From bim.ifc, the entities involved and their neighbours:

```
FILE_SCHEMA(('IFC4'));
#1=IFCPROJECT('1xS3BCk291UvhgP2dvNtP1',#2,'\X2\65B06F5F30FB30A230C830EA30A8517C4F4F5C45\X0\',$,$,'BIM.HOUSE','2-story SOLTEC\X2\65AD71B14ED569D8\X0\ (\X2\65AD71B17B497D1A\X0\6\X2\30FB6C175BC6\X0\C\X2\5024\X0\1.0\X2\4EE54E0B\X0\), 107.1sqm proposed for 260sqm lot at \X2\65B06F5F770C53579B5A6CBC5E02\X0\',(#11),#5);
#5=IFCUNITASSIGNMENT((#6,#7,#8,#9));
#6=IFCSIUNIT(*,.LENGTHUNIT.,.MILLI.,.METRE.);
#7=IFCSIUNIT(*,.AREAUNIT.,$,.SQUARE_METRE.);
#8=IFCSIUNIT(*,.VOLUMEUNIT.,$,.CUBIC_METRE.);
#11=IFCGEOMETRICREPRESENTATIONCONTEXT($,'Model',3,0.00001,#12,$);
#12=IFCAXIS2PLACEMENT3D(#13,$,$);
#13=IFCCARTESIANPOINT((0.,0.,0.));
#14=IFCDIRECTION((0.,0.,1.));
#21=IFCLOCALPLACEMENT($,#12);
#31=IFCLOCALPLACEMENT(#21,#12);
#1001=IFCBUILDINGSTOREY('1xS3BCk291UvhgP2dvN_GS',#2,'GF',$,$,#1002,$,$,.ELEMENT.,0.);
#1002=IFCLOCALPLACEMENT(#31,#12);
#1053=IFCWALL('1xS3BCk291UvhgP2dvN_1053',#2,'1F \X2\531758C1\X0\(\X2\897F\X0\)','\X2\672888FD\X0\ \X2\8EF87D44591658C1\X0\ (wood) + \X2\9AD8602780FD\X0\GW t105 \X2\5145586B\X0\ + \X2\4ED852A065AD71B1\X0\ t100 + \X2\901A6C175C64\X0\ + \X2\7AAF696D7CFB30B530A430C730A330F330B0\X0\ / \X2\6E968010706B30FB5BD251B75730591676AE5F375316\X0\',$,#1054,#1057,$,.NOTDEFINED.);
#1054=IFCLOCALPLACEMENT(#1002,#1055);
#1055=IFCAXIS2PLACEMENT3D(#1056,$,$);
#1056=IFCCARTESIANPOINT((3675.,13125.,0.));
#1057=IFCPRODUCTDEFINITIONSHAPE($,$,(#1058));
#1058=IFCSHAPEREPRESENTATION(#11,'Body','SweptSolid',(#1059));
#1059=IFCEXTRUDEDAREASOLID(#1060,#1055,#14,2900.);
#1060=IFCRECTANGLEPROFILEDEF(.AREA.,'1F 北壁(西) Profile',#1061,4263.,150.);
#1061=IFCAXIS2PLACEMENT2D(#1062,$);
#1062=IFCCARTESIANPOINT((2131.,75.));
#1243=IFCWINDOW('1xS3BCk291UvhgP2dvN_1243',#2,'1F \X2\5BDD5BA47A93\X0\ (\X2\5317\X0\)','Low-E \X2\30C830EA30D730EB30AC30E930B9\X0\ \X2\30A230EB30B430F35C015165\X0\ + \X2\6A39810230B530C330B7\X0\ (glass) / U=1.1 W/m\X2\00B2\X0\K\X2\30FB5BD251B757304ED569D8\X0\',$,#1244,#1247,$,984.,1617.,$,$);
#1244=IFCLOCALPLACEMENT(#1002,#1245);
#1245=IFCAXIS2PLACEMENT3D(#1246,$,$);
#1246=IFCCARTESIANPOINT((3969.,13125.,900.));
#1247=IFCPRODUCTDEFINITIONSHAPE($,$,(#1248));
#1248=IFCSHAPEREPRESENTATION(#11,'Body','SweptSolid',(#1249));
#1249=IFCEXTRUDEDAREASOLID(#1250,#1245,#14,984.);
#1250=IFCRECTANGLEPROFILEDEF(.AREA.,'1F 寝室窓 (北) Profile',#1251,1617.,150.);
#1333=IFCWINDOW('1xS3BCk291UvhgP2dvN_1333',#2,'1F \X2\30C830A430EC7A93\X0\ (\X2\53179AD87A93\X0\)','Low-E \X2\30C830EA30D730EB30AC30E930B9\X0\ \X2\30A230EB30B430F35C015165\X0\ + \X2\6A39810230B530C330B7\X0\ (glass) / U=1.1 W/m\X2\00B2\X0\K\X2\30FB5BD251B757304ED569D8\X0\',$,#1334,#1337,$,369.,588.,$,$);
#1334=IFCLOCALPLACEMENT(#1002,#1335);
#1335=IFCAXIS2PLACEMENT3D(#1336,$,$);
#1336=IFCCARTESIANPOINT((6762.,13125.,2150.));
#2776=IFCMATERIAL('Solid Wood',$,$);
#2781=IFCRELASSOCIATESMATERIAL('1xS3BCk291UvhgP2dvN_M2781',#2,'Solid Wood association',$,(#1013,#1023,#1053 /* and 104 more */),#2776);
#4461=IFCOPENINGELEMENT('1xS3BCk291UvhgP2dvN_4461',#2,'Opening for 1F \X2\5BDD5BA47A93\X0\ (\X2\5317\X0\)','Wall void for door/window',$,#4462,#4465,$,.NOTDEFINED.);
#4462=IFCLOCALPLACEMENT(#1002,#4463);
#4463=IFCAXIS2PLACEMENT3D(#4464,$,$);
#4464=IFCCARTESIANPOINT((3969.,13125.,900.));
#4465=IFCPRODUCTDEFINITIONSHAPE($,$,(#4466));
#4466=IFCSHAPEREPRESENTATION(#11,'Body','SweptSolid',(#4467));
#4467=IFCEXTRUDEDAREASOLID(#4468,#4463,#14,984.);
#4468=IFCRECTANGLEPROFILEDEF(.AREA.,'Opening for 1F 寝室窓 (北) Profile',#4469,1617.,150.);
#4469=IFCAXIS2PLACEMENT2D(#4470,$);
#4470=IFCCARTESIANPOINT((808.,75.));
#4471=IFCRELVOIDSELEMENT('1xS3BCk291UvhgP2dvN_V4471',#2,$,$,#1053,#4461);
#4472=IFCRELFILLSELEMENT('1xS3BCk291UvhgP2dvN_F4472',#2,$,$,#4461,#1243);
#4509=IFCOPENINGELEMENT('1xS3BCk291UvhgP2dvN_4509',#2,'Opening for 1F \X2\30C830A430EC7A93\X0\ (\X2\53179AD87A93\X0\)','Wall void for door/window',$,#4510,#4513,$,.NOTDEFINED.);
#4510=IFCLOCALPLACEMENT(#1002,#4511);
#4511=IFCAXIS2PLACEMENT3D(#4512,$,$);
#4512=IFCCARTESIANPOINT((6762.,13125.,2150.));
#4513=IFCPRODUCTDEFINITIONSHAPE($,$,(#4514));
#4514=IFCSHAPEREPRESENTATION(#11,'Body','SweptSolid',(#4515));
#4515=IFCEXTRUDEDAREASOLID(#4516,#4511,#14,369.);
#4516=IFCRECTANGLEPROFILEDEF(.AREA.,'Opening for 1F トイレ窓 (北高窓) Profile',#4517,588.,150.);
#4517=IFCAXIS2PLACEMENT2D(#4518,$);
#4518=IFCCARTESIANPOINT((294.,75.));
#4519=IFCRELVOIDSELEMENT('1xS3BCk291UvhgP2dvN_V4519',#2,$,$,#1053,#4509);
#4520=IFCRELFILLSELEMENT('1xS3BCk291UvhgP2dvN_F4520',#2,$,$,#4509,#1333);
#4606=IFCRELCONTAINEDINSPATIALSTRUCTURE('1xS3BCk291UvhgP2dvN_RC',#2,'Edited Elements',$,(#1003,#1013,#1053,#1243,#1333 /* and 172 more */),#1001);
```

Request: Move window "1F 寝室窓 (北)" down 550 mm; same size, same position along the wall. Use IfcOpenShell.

```python
import numpy as np
import ifcopenshell
import ifcopenshell.api.geometry
import ifcopenshell.util.placement
import ifcopenshell.util.unit

model = ifcopenshell.open("bim.ifc")
unit_scale = ifcopenshell.util.unit.calculate_unit_scale(model)

window = model.by_guid("1xS3BCk291UvhgP2dvN_1243")
opening = window.FillsVoids[0].RelatingOpeningElement
dz = -0.55 / unit_scale

shift = np.array([0.0, 0.0, dz])
# The window is not placed relative to its opening, so move both.
for product in (opening, window):
    matrix = ifcopenshell.util.placement.get_local_placement(product.ObjectPlacement)
    matrix[:3, 3] += shift
    ifcopenshell.api.geometry.edit_object_placement(model, product=product, matrix=matrix, is_si=False)

print(f"moved by {dz * unit_scale:+.3f} m")

model.write("bim_updated.ifc")
```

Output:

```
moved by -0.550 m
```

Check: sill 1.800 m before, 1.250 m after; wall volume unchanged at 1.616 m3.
